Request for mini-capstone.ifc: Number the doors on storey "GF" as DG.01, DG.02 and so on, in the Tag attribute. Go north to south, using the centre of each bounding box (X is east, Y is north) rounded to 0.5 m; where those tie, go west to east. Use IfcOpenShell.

First a look at what the model holds.

```python
import ifcopenshell
import ifcopenshell.util.element
import ifcopenshell.util.placement

model = ifcopenshell.open("mini-capstone.ifc")
print(model.schema)
storey = next(s for s in model.by_type("IfcBuildingStorey") if s.Name == "GF")
doors = [e for e in ifcopenshell.util.element.get_decomposition(storey) if e.is_a("IfcDoor")]
for e in sorted(doors, key=lambda e: e.id()):
    origin = ifcopenshell.util.placement.get_local_placement(e.ObjectPlacement)[:3, 3]
    print(e.id(), e.Tag, e.Name, origin.round(2) + 0.0, sep=" | ")
```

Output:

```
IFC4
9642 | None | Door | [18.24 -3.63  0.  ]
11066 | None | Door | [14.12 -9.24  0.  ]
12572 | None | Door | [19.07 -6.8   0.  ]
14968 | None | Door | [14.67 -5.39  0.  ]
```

```python
import ifcopenshell
import ifcopenshell.geom
import ifcopenshell.util.element
import ifcopenshell.util.shape

model = ifcopenshell.open("mini-capstone.ifc")
settings = ifcopenshell.geom.settings()
settings.set("use-world-coords", True)


def centre(element):
    shape = ifcopenshell.geom.create_shape(settings, element)
    return ifcopenshell.util.shape.get_bbox_centroid(shape.geometry)


storey = next(s for s in model.by_type("IfcBuildingStorey") if s.Name == "GF")
doors = [e for e in ifcopenshell.util.element.get_decomposition(storey) if e.is_a("IfcDoor")]

# Insertion points can sit at a corner or the storey origin, so sort by the geometry (in metres).
centres = {e: centre(e) for e in doors}
doors.sort(key=lambda e: (-round(centres[e][1] / 0.5), centres[e][0]))

for i, e in enumerate(doors, start=1):
    number = f"DG.{i:02d}"
    e.Tag = number
    print(e.id(), number)

model.write("mini-capstone_v2.ifc")
```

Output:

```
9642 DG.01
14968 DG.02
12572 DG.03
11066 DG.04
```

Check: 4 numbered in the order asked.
